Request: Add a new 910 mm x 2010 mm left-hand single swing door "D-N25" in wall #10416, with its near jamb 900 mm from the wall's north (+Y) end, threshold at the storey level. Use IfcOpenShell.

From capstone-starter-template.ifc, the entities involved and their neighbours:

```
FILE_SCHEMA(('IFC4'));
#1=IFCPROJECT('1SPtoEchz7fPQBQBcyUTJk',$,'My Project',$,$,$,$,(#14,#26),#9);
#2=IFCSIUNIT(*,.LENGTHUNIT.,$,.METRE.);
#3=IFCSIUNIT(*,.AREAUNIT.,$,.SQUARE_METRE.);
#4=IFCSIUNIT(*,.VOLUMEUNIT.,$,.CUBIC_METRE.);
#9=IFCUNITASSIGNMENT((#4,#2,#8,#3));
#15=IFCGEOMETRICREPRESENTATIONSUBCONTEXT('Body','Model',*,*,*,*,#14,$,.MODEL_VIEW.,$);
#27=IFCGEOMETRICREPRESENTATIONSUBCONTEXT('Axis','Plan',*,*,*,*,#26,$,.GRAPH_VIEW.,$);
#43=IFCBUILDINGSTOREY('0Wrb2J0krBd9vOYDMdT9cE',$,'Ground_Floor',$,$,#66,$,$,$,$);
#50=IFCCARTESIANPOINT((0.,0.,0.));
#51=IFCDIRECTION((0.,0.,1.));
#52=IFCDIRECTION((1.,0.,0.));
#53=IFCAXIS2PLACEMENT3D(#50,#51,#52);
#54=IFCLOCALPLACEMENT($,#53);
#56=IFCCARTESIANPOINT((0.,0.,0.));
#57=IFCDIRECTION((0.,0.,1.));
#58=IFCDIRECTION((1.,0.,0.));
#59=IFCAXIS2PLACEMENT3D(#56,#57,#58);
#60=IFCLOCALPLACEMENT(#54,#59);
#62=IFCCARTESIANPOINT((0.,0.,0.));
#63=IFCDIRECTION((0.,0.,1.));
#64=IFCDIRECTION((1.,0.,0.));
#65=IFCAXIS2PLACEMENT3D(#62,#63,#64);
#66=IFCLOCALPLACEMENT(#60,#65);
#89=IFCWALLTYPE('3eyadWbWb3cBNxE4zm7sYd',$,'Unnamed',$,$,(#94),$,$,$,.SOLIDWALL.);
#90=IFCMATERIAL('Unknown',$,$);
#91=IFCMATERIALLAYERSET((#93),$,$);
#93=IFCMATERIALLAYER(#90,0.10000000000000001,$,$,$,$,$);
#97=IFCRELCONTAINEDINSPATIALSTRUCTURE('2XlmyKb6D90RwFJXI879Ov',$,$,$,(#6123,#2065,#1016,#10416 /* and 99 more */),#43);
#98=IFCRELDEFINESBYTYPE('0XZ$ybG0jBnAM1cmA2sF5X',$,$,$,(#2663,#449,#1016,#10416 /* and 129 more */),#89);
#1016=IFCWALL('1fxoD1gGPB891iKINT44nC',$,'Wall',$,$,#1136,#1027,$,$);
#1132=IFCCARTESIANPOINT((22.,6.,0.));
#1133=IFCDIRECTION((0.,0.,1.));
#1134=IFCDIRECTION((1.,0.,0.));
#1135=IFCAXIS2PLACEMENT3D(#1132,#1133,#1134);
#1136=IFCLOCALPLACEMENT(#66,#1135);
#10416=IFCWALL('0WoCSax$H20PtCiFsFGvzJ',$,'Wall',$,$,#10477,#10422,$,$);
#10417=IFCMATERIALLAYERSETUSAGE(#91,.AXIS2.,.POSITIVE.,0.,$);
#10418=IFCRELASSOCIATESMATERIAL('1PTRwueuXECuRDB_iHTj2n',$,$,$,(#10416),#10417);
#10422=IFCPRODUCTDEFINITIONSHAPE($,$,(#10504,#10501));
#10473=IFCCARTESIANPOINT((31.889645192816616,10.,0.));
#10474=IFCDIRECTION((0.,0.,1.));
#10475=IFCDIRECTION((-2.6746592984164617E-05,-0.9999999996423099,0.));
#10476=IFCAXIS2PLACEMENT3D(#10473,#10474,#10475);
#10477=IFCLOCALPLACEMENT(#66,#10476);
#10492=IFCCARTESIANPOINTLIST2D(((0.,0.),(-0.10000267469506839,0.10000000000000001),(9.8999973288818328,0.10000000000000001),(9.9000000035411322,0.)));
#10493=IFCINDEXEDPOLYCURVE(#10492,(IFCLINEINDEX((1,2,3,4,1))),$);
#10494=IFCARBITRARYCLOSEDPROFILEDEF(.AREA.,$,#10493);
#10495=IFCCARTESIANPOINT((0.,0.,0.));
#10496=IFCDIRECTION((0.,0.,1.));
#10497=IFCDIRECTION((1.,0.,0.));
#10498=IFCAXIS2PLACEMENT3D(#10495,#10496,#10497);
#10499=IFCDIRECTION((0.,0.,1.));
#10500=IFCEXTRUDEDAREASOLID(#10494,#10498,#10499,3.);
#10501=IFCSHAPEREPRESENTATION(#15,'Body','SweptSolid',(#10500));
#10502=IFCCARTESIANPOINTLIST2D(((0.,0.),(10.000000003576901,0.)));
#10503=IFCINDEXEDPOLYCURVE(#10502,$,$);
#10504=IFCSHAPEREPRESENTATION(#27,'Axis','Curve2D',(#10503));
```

```python
import numpy as np
import ifcopenshell
import ifcopenshell.api.feature
import ifcopenshell.api.geometry
import ifcopenshell.api.root
import ifcopenshell.api.spatial
import ifcopenshell.geom
import ifcopenshell.util.element
import ifcopenshell.util.placement
import ifcopenshell.util.representation
import ifcopenshell.util.shape
import ifcopenshell.util.unit

model = ifcopenshell.open("capstone-starter-template.ifc")
unit_scale = ifcopenshell.util.unit.calculate_unit_scale(model)
settings = ifcopenshell.geom.settings()


def volume(element):
    """Net volume in cubic metres, openings subtracted."""
    shape = ifcopenshell.geom.create_shape(settings, element)
    return ifcopenshell.util.shape.get_volume(shape.geometry)


wall = model.by_guid("0WoCSax$H20PtCiFsFGvzJ")
storey = ifcopenshell.util.element.get_container(wall, ifc_class="IfcBuildingStorey")
context = ifcopenshell.util.representation.get_context(model, "Model", "Body", "MODEL_VIEW")
before = volume(wall)

width, height, from_end, sill = 0.91, 2.01, 0.9, 0.0  # metres

# The wall runs along its own X axis, and the end named is its -X end.
wall_shape = ifcopenshell.geom.create_shape(settings, wall)
x, y, z = ifcopenshell.util.shape.get_vertices(wall_shape.geometry).T
start = x.min() + from_end
face, thickness = float(y.min()), float(y.max() - y.min())
wall_matrix = ifcopenshell.util.placement.get_local_placement(wall.ObjectPlacement)
level = ifcopenshell.util.placement.get_local_placement(storey.ObjectPlacement)[2, 3]


def in_wall(x, y):
    """Placement at x, y metres in the wall's axes, at sill height."""
    matrix = wall_matrix.copy()
    matrix[:, 3] = wall_matrix @ np.array([x / unit_scale, y / unit_scale, 0.0, 1.0])
    matrix[2, 3] = level + sill / unit_scale
    return matrix


# Opening: a box that overshoots both wall faces by 50 mm.
opening = ifcopenshell.api.root.create_entity(model, ifc_class="IfcOpeningElement", predefined_type="OPENING")
box = ifcopenshell.api.geometry.add_wall_representation(
    model, context=context, length=width, height=height, thickness=thickness + 0.1
)
ifcopenshell.api.geometry.assign_representation(model, product=opening, representation=box)
ifcopenshell.api.geometry.edit_object_placement(model, product=opening, matrix=in_wall(start, face - 0.05), is_si=False)
ifcopenshell.api.feature.add_feature(model, feature=opening, element=wall)

door = ifcopenshell.api.root.create_entity(model, ifc_class="IfcDoor", name="D-N25", predefined_type="DOOR")
door.OverallWidth, door.OverallHeight = width / unit_scale, height / unit_scale
door.OperationType = "SINGLE_SWING_LEFT"
body = ifcopenshell.api.geometry.add_door_representation(
    model,
    context=context,
    overall_width=door.OverallWidth,
    overall_height=door.OverallHeight,
    operation_type="SINGLE_SWING_LEFT",
    lining_properties={"LiningDepth": thickness / unit_scale, "ThresholdDepth": thickness / unit_scale},
)
ifcopenshell.api.geometry.assign_representation(model, product=door, representation=body)
ifcopenshell.api.spatial.assign_container(model, products=[door], relating_structure=storey)
ifcopenshell.api.feature.add_filling(model, opening=opening, element=door)

# The lining spans the wall, so the door starts at the wall face.
ifcopenshell.api.geometry.edit_object_placement(model, product=door, matrix=in_wall(start, face), is_si=False)

after = volume(wall)

print(f"wall volume {before:.3f} -> {after:.3f} m3")

model.write("capstone-starter-template_rev.ifc")
```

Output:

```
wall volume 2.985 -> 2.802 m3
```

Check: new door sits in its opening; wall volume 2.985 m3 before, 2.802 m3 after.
